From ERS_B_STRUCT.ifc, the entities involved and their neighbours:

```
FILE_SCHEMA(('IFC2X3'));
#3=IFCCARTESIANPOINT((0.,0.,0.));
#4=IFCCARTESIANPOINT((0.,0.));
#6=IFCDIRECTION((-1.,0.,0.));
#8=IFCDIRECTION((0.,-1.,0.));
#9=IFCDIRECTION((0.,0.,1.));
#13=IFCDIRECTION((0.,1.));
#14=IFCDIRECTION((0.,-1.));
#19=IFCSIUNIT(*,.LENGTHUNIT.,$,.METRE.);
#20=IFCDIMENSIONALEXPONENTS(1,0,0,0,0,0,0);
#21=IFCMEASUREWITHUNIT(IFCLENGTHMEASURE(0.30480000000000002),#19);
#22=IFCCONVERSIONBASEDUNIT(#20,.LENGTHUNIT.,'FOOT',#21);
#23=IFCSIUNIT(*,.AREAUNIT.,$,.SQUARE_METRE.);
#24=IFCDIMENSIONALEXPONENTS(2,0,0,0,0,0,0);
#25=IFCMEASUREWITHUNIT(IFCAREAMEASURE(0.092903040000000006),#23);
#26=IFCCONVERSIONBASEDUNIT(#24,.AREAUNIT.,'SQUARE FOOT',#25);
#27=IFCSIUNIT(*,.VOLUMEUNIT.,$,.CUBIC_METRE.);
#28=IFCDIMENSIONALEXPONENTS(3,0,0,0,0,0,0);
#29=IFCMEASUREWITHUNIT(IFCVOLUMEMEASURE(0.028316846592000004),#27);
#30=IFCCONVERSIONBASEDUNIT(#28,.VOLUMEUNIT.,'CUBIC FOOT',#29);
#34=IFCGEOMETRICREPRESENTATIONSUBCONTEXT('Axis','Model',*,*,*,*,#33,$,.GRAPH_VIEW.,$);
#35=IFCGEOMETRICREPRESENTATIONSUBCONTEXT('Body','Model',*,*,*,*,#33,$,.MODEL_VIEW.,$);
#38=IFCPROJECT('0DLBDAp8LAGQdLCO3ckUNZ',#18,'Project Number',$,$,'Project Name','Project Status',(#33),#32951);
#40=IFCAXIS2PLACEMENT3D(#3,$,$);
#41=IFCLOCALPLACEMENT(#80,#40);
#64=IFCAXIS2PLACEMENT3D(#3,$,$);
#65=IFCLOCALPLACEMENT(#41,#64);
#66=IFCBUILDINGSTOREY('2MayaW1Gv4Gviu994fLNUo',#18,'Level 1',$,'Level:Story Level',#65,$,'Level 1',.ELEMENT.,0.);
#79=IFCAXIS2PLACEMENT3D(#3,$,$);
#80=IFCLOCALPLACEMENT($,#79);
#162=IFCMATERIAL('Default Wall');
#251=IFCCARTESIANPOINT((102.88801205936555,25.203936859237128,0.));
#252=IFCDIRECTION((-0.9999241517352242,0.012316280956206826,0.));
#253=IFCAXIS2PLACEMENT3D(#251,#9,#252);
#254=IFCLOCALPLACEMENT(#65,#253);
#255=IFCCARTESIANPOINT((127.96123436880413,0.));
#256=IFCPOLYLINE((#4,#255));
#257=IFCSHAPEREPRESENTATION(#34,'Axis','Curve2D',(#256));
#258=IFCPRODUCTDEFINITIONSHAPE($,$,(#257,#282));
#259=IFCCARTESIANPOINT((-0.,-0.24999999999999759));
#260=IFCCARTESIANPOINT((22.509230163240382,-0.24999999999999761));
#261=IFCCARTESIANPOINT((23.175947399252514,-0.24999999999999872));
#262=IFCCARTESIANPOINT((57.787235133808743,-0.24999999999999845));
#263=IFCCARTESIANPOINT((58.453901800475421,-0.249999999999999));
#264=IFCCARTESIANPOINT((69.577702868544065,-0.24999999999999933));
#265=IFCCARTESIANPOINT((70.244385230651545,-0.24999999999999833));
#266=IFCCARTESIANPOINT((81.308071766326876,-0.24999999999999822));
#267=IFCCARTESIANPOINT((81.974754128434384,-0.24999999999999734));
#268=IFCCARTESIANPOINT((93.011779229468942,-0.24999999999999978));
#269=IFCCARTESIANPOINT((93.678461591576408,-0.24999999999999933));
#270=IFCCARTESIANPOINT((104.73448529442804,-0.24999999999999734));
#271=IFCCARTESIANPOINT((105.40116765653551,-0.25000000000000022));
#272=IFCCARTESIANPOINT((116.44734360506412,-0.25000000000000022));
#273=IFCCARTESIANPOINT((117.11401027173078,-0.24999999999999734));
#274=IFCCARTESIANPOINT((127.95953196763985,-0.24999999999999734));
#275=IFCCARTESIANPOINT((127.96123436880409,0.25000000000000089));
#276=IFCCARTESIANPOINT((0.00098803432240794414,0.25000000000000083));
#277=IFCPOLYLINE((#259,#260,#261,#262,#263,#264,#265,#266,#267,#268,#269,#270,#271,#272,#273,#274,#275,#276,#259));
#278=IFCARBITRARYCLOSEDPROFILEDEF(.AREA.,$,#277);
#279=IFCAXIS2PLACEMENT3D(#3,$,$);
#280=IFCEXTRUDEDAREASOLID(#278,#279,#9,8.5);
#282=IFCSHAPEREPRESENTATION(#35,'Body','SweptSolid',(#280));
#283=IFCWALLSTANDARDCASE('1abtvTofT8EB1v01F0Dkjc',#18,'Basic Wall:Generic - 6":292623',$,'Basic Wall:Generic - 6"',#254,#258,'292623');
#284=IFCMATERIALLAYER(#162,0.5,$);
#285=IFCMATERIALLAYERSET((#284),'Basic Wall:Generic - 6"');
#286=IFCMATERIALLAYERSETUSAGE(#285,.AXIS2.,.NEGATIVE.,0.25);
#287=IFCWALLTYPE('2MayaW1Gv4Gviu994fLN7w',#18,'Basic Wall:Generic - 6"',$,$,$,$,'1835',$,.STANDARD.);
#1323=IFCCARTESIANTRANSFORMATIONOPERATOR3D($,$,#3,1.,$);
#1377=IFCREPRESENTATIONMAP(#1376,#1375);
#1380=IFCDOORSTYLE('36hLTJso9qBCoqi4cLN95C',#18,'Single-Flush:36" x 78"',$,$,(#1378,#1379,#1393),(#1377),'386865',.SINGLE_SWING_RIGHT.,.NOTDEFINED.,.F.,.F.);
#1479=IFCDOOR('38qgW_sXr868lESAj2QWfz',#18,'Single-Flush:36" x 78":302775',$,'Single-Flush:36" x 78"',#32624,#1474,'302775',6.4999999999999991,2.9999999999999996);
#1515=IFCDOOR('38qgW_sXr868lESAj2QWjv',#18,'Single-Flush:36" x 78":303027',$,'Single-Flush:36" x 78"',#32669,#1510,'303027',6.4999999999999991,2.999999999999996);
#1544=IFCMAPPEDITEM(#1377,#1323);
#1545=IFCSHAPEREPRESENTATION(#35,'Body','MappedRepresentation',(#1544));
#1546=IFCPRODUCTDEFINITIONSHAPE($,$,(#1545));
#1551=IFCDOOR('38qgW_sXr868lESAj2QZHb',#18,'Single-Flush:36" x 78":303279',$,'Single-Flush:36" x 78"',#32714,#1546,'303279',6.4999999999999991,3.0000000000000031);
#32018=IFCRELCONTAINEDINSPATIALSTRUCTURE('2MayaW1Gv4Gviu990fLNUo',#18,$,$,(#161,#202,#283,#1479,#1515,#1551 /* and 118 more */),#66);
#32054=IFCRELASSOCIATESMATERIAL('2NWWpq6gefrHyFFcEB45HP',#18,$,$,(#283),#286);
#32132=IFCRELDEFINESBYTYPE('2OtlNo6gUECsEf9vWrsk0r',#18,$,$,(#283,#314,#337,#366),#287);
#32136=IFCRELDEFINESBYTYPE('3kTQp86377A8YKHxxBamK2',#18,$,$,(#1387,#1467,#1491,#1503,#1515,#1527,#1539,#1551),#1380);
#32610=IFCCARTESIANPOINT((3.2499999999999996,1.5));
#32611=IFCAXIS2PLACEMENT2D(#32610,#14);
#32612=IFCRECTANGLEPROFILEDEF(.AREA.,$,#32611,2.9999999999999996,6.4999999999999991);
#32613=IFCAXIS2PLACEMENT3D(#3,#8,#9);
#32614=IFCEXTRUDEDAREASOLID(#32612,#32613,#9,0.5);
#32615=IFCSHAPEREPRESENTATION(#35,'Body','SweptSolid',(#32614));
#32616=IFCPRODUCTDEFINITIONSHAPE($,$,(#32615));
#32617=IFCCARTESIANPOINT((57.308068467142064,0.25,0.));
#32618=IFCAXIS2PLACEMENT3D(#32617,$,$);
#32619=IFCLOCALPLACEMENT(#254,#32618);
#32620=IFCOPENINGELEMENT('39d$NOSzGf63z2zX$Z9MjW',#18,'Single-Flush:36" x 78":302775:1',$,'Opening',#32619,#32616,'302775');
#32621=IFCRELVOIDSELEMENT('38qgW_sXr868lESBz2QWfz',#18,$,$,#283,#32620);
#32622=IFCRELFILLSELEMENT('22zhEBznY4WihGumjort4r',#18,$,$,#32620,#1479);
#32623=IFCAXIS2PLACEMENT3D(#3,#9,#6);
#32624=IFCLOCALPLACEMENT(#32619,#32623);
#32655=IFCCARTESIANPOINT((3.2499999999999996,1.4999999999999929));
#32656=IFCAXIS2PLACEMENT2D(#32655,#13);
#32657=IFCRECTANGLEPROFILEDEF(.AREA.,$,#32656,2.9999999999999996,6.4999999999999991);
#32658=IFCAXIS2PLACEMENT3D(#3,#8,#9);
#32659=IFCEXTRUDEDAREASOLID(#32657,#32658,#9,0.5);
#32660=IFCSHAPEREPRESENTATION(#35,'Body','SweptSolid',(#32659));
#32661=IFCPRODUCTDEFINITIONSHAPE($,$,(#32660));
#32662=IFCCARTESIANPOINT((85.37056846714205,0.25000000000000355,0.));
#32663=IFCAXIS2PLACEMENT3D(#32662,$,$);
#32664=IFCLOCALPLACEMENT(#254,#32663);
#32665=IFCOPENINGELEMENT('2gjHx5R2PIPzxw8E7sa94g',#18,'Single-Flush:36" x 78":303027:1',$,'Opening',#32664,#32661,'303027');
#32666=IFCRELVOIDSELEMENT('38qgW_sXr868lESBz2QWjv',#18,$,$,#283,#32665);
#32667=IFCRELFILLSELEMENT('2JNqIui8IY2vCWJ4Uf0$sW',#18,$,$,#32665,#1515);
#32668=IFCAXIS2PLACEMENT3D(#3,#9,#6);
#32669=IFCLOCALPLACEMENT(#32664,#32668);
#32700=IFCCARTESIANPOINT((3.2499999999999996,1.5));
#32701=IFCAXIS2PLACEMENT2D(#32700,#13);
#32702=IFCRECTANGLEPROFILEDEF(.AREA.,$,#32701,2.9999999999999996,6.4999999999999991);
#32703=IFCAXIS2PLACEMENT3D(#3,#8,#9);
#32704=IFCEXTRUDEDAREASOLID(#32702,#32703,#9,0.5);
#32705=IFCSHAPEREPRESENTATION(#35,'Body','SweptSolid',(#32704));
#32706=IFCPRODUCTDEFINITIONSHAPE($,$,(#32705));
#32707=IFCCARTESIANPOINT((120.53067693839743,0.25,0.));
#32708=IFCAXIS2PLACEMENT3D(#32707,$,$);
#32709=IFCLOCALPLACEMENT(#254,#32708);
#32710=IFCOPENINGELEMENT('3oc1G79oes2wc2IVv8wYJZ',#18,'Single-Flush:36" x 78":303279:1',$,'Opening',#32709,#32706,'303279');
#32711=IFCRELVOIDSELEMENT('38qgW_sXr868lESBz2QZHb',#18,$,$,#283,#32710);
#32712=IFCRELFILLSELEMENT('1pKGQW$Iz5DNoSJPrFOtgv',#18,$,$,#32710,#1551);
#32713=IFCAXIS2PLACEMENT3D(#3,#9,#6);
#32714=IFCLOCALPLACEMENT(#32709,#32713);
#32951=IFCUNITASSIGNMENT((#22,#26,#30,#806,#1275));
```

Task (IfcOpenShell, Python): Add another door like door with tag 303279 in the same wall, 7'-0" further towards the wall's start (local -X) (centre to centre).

```python
import ifcopenshell
import ifcopenshell.api.feature
import ifcopenshell.api.geometry
import ifcopenshell.api.root
import ifcopenshell.geom
import ifcopenshell.util.element
import ifcopenshell.util.placement
import ifcopenshell.util.shape
import ifcopenshell.util.unit

model = ifcopenshell.open("ERS_B_STRUCT.ifc")
unit_scale = ifcopenshell.util.unit.calculate_unit_scale(model)
settings = ifcopenshell.geom.settings()


def volume(element):
    """Net volume in cubic metres, openings subtracted."""
    shape = ifcopenshell.geom.create_shape(settings, element)
    return ifcopenshell.util.shape.get_volume(shape.geometry)


def reuse_history(source, copy):
    """copy_class also copies each property set's owner history, people and application; keep the originals."""
    for rel in copy.IsDefinedBy:
        if rel.is_a("IfcRelDefinesByProperties") and (history := rel.RelatingPropertyDefinition.OwnerHistory):
            rel.RelatingPropertyDefinition.OwnerHistory = source.OwnerHistory
            ifcopenshell.util.element.remove_deep2(model, history)


door = model.by_guid("38qgW_sXr868lESAj2QZHb")
opening = door.FillsVoids[0].RelatingOpeningElement
wall = opening.VoidsElements[0].RelatingBuildingElement
before = volume(wall)
shift = ifcopenshell.util.placement.get_local_placement(wall.ObjectPlacement)[:3, 0] * -84 * 0.0254 / unit_scale

# copy_class copies the void relationship, type, container and properties, but no geometry.
new_opening = ifcopenshell.api.root.copy_class(model, product=opening)
new_opening.Representation = ifcopenshell.util.element.copy_deep(
    model, opening.Representation, exclude=["IfcGeometricRepresentationContext", "IfcRepresentationMap"]
)
new_opening.Name = 'Single-Flush:36" x 78"'
new_opening.Tag = None
new_door = ifcopenshell.api.root.copy_class(model, product=door)
new_door.Representation = ifcopenshell.util.element.copy_deep(
    model, door.Representation, exclude=["IfcGeometricRepresentationContext", "IfcRepresentationMap"]
)
new_door.Name = 'Single-Flush:36" x 78"'
new_door.Tag = None
reuse_history(door, new_door)
fills = ifcopenshell.api.feature.add_filling(model, opening=new_opening, element=new_door)
fills.OwnerHistory = new_door.OwnerHistory  # required in IFC2X3

for old, new in ((opening, new_opening), (door, new_door)):
    matrix = ifcopenshell.util.placement.get_local_placement(old.ObjectPlacement)
    matrix[:3, 3] += shift
    ifcopenshell.api.geometry.edit_object_placement(model, product=new, matrix=matrix, is_si=False)

after = volume(wall)

print(f"wall volume {before:.3f} -> {after:.3f} m3")

model.write("ERS_B_STRUCT_v2.ifc")
```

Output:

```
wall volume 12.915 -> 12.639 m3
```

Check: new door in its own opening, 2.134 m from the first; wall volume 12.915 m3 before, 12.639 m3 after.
